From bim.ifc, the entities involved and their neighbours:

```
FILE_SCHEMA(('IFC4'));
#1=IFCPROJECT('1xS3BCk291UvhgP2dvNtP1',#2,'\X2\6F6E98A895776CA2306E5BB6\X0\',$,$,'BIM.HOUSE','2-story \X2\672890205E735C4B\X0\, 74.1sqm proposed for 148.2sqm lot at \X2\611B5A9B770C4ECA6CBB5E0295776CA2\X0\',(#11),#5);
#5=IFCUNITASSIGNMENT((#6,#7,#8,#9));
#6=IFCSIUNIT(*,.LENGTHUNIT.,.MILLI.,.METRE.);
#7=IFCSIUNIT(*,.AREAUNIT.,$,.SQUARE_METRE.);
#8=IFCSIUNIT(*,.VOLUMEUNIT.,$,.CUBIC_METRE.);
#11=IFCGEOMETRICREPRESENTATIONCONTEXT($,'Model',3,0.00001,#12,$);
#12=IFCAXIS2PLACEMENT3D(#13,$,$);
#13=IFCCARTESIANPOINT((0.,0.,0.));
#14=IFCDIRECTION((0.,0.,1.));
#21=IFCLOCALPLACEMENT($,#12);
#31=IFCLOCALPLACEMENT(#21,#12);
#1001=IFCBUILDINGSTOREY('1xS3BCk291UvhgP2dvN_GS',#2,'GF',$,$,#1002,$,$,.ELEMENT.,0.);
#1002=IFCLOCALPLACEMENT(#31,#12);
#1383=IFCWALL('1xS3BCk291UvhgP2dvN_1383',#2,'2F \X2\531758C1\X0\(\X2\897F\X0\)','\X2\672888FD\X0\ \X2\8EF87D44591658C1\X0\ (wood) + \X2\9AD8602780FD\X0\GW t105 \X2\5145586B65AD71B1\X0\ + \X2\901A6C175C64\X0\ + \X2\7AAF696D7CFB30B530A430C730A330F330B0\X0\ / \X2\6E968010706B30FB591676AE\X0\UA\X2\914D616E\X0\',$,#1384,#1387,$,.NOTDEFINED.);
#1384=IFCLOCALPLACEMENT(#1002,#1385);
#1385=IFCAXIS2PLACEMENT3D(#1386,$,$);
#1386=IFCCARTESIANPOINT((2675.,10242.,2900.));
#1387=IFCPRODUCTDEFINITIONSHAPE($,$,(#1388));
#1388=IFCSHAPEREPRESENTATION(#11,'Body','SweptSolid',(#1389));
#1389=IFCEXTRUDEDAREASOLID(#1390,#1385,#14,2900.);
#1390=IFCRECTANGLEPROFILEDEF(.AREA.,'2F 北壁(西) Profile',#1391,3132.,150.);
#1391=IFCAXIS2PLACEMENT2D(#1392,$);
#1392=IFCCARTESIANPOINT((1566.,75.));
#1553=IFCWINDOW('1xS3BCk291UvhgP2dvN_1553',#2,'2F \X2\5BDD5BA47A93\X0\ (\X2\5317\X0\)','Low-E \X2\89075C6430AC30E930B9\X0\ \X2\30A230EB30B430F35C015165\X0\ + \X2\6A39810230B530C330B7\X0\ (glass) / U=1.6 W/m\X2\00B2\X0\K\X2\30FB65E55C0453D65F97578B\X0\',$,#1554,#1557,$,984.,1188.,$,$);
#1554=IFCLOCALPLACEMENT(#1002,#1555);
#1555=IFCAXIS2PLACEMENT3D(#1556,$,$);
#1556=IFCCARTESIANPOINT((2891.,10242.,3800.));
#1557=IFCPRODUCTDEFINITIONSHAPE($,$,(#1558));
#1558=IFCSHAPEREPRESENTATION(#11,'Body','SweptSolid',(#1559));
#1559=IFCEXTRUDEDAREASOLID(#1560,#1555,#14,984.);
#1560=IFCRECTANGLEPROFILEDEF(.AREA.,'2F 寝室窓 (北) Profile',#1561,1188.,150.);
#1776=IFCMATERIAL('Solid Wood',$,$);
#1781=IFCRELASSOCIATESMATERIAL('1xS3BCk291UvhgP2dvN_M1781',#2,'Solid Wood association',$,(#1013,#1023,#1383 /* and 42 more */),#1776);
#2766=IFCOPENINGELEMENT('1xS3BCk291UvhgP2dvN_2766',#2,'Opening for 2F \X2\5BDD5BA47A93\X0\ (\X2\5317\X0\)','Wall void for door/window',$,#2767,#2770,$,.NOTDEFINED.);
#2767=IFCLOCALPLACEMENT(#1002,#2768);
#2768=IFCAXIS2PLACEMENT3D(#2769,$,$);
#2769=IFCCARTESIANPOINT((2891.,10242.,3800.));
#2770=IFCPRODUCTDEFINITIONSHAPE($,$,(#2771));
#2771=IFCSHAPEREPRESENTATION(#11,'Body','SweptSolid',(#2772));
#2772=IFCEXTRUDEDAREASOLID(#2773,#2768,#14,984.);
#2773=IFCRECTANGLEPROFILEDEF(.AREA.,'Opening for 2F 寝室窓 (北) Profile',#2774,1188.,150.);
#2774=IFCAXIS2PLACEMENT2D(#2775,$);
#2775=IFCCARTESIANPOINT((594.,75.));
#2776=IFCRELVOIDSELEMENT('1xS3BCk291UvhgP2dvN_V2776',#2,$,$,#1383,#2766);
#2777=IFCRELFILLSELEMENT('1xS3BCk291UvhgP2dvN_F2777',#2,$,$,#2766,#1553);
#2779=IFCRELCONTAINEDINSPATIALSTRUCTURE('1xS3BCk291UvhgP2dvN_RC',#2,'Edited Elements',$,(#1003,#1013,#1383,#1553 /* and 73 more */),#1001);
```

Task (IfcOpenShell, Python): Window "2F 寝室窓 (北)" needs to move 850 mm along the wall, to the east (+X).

```python
import ifcopenshell
import ifcopenshell.api.geometry
import ifcopenshell.util.placement
import ifcopenshell.util.unit

model = ifcopenshell.open("bim.ifc")
unit_scale = ifcopenshell.util.unit.calculate_unit_scale(model)

window = model.by_guid("1xS3BCk291UvhgP2dvN_1553")
opening = window.FillsVoids[0].RelatingOpeningElement
wall = opening.VoidsElements[0].RelatingBuildingElement

wall_matrix = ifcopenshell.util.placement.get_local_placement(wall.ObjectPlacement)
shift = wall_matrix[:3, 0] * 0.85 / unit_scale
before = ifcopenshell.util.placement.get_local_placement(window.ObjectPlacement)[:3, 3].copy()

# The window is not placed relative to its opening, so move both.
for product in (opening, window):
    matrix = ifcopenshell.util.placement.get_local_placement(product.ObjectPlacement)
    matrix[:3, 3] += shift
    ifcopenshell.api.geometry.edit_object_placement(model, product=product, matrix=matrix, is_si=False)

after = ifcopenshell.util.placement.get_local_placement(window.ObjectPlacement)[:3, 3]
print("window moved by", (after - before).round(3) + 0.0)

model.write("bim-out.ifc")
```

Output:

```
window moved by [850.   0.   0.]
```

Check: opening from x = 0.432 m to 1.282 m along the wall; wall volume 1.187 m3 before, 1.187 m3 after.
